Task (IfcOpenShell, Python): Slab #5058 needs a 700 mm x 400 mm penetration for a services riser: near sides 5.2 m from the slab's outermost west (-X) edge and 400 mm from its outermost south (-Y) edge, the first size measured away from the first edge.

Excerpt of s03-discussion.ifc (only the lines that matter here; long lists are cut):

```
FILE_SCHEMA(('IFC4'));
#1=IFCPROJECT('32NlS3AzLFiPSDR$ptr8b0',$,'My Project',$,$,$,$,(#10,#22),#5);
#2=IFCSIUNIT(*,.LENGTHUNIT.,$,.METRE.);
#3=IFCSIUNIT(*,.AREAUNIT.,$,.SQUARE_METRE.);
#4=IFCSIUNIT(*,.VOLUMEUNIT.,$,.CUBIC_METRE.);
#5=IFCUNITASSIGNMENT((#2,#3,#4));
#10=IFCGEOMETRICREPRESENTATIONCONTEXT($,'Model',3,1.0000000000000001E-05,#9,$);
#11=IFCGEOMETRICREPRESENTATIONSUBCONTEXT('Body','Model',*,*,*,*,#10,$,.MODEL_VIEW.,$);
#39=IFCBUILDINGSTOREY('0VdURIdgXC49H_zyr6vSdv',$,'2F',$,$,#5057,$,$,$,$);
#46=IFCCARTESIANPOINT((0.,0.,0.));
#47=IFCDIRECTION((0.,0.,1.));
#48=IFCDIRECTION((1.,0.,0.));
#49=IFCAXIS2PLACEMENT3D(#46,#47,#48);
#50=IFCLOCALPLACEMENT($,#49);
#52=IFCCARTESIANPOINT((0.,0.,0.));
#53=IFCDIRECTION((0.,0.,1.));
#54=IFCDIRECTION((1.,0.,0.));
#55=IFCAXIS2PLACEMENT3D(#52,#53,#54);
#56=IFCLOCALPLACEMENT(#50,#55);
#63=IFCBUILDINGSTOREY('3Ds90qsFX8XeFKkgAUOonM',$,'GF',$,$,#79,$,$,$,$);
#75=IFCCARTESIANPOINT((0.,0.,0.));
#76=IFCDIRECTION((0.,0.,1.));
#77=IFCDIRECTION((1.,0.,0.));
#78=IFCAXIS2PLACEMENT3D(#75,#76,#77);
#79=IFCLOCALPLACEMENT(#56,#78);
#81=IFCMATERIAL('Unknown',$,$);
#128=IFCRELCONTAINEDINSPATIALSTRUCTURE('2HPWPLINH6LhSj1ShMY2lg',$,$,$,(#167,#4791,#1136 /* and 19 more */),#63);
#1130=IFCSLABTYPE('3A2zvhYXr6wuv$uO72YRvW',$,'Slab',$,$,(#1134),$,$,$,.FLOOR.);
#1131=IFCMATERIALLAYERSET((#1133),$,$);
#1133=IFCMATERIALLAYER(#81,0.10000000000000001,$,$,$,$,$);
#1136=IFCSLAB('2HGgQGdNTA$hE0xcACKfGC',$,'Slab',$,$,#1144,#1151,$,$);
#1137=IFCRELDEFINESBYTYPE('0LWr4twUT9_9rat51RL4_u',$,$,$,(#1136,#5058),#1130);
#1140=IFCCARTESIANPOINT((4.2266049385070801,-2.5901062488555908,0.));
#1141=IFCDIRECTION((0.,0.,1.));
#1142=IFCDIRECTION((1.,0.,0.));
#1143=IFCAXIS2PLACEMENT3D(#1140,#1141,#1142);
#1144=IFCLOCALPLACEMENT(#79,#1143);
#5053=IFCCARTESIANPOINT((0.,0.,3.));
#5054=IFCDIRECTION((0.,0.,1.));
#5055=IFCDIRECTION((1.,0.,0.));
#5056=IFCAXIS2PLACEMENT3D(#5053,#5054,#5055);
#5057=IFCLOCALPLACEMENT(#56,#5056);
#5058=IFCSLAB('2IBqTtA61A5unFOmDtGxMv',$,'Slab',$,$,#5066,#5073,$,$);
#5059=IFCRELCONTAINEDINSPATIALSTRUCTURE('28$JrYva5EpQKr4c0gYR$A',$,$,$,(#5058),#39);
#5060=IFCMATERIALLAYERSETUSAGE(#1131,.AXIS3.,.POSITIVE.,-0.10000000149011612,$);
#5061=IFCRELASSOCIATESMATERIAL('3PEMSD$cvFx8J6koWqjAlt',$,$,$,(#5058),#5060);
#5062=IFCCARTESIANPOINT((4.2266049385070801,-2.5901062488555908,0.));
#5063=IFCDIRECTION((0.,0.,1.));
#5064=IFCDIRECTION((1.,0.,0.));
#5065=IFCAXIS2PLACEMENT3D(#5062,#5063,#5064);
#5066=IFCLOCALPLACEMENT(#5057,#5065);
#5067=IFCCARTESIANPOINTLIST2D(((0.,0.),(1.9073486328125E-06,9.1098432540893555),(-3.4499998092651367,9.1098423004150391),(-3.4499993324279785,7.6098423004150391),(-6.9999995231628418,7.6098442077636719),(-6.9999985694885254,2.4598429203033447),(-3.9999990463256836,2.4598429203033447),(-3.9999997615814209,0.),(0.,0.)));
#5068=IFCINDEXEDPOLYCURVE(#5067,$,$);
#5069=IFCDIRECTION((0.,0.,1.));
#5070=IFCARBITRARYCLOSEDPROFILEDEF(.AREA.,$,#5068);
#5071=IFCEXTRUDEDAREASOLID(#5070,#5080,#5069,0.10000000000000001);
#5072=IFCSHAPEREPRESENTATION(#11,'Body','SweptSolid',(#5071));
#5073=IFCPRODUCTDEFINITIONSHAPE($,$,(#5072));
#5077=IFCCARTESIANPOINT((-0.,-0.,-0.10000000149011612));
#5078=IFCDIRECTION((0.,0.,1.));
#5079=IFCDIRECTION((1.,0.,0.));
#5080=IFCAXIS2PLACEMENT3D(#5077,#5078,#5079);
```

```python
import numpy as np
import ifcopenshell
import ifcopenshell.api.feature
import ifcopenshell.api.geometry
import ifcopenshell.api.root
import ifcopenshell.geom
import ifcopenshell.util.placement
import ifcopenshell.util.representation
import ifcopenshell.util.shape
import ifcopenshell.util.unit

model = ifcopenshell.open("s03-discussion.ifc")
unit_scale = ifcopenshell.util.unit.calculate_unit_scale(model)
settings = ifcopenshell.geom.settings()


def volume(element):
    """Net volume in cubic metres, openings subtracted."""
    shape = ifcopenshell.geom.create_shape(settings, element)
    return ifcopenshell.util.shape.get_volume(shape.geometry)


slab = model.by_guid("2IBqTtA61A5unFOmDtGxMv")
before = volume(slab)

# Extent in the slab's own axes, in metres. The edges named are its -X and -Y sides.
slab_shape = ifcopenshell.geom.create_shape(settings, slab)
vertices = ifcopenshell.util.shape.get_vertices(slab_shape.geometry)
x_min, y_min, bottom = vertices.min(axis=0)
top = vertices[:, 2].max()

opening = ifcopenshell.api.root.create_entity(model, ifc_class="IfcOpeningElement", name="Services riser opening", predefined_type="OPENING")
context = ifcopenshell.util.representation.get_context(model, "Model", "Body", "MODEL_VIEW")
width, depth = 0.7, 0.4
outline = [(0.0, 0.0), (width, 0.0), (width, depth), (0.0, depth), (0.0, 0.0)]
# Overshoot both faces by 50 mm so the cut is clean.
shape = ifcopenshell.api.geometry.add_slab_representation(
    model, context=context, depth=top - bottom + 0.1, polyline=outline
)
ifcopenshell.api.geometry.assign_representation(model, product=opening, representation=shape)

matrix = ifcopenshell.util.placement.get_local_placement(slab.ObjectPlacement)
matrix[:, 3] = matrix @ np.append(np.array([x_min + 5.2, y_min + 0.4, bottom - 0.05]) / unit_scale, 1.0)
ifcopenshell.api.geometry.edit_object_placement(model, product=opening, matrix=matrix, is_si=False)
ifcopenshell.api.feature.add_feature(model, feature=opening, element=slab)

after = volume(slab)

print(f"slab volume {before:.3f} -> {after:.3f} m3")

model.write("s03-discussion_edited.ifc")
```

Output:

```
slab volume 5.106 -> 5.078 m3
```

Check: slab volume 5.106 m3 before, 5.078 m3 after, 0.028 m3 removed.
